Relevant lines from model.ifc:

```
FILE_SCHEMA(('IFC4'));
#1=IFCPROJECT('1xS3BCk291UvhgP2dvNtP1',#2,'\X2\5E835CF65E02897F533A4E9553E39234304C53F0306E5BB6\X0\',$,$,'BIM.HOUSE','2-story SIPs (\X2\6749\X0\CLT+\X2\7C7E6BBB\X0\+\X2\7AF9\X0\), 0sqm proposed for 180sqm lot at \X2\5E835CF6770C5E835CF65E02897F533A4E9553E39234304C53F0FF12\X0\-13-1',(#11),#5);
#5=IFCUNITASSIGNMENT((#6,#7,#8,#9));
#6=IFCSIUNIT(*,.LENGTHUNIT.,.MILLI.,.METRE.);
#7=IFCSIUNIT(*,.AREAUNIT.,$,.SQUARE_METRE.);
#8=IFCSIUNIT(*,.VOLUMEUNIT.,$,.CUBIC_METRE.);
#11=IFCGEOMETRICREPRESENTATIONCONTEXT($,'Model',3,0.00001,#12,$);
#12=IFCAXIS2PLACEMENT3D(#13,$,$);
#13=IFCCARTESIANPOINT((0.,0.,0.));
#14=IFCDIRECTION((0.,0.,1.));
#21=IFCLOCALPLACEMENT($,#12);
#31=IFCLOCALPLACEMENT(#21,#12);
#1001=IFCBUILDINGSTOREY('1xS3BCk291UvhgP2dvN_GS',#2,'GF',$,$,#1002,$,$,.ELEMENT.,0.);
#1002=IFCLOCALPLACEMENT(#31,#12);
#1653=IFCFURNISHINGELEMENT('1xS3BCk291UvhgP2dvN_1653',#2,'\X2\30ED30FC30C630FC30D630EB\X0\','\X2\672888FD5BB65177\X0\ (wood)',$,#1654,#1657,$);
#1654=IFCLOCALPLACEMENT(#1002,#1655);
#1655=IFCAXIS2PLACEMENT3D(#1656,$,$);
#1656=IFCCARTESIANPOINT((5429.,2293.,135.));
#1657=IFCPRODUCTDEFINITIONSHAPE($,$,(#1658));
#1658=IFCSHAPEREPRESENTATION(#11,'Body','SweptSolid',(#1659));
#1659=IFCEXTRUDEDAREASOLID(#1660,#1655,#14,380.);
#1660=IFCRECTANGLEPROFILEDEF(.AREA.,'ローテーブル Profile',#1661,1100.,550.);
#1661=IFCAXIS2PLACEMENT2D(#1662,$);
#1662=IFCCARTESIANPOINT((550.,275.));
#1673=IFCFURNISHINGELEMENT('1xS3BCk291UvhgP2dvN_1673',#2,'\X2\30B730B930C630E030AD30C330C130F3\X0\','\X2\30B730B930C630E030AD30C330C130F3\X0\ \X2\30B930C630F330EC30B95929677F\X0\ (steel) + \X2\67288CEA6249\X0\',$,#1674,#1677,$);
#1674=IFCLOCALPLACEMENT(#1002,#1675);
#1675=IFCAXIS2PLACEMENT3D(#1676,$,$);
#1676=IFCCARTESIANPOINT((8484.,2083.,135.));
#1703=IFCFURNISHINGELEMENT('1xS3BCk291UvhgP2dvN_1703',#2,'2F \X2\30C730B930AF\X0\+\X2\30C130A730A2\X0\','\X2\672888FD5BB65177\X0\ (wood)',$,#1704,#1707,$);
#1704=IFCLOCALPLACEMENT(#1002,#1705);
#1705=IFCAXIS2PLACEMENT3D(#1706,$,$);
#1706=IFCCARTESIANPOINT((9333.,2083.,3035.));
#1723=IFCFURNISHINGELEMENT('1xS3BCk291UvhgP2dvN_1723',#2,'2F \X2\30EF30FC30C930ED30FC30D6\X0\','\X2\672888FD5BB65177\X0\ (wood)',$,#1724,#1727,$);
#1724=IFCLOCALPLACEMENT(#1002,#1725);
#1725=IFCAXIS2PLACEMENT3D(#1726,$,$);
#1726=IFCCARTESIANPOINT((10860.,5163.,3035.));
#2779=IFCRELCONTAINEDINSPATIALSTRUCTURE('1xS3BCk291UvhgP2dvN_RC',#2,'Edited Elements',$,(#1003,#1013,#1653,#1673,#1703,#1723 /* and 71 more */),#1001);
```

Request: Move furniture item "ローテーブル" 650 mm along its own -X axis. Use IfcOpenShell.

```python
import ifcopenshell
import ifcopenshell.api.geometry
import ifcopenshell.util.placement

model = ifcopenshell.open("model.ifc")

item = model.by_guid("1xS3BCk291UvhgP2dvN_1653")
matrix = ifcopenshell.util.placement.get_local_placement(item.ObjectPlacement)
matrix[:3, 3] -= matrix[:3, 0] * 650.0
ifcopenshell.api.geometry.edit_object_placement(model, product=item, matrix=matrix, is_si=False)

print(ifcopenshell.util.placement.get_local_placement(item.ObjectPlacement).round(3) + 0.0)

model.write("model_v2.ifc")
```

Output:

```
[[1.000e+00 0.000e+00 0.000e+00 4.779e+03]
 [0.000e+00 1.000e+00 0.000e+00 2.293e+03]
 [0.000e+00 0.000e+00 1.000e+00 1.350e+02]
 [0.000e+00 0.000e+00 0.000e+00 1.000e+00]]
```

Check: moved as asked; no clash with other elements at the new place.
